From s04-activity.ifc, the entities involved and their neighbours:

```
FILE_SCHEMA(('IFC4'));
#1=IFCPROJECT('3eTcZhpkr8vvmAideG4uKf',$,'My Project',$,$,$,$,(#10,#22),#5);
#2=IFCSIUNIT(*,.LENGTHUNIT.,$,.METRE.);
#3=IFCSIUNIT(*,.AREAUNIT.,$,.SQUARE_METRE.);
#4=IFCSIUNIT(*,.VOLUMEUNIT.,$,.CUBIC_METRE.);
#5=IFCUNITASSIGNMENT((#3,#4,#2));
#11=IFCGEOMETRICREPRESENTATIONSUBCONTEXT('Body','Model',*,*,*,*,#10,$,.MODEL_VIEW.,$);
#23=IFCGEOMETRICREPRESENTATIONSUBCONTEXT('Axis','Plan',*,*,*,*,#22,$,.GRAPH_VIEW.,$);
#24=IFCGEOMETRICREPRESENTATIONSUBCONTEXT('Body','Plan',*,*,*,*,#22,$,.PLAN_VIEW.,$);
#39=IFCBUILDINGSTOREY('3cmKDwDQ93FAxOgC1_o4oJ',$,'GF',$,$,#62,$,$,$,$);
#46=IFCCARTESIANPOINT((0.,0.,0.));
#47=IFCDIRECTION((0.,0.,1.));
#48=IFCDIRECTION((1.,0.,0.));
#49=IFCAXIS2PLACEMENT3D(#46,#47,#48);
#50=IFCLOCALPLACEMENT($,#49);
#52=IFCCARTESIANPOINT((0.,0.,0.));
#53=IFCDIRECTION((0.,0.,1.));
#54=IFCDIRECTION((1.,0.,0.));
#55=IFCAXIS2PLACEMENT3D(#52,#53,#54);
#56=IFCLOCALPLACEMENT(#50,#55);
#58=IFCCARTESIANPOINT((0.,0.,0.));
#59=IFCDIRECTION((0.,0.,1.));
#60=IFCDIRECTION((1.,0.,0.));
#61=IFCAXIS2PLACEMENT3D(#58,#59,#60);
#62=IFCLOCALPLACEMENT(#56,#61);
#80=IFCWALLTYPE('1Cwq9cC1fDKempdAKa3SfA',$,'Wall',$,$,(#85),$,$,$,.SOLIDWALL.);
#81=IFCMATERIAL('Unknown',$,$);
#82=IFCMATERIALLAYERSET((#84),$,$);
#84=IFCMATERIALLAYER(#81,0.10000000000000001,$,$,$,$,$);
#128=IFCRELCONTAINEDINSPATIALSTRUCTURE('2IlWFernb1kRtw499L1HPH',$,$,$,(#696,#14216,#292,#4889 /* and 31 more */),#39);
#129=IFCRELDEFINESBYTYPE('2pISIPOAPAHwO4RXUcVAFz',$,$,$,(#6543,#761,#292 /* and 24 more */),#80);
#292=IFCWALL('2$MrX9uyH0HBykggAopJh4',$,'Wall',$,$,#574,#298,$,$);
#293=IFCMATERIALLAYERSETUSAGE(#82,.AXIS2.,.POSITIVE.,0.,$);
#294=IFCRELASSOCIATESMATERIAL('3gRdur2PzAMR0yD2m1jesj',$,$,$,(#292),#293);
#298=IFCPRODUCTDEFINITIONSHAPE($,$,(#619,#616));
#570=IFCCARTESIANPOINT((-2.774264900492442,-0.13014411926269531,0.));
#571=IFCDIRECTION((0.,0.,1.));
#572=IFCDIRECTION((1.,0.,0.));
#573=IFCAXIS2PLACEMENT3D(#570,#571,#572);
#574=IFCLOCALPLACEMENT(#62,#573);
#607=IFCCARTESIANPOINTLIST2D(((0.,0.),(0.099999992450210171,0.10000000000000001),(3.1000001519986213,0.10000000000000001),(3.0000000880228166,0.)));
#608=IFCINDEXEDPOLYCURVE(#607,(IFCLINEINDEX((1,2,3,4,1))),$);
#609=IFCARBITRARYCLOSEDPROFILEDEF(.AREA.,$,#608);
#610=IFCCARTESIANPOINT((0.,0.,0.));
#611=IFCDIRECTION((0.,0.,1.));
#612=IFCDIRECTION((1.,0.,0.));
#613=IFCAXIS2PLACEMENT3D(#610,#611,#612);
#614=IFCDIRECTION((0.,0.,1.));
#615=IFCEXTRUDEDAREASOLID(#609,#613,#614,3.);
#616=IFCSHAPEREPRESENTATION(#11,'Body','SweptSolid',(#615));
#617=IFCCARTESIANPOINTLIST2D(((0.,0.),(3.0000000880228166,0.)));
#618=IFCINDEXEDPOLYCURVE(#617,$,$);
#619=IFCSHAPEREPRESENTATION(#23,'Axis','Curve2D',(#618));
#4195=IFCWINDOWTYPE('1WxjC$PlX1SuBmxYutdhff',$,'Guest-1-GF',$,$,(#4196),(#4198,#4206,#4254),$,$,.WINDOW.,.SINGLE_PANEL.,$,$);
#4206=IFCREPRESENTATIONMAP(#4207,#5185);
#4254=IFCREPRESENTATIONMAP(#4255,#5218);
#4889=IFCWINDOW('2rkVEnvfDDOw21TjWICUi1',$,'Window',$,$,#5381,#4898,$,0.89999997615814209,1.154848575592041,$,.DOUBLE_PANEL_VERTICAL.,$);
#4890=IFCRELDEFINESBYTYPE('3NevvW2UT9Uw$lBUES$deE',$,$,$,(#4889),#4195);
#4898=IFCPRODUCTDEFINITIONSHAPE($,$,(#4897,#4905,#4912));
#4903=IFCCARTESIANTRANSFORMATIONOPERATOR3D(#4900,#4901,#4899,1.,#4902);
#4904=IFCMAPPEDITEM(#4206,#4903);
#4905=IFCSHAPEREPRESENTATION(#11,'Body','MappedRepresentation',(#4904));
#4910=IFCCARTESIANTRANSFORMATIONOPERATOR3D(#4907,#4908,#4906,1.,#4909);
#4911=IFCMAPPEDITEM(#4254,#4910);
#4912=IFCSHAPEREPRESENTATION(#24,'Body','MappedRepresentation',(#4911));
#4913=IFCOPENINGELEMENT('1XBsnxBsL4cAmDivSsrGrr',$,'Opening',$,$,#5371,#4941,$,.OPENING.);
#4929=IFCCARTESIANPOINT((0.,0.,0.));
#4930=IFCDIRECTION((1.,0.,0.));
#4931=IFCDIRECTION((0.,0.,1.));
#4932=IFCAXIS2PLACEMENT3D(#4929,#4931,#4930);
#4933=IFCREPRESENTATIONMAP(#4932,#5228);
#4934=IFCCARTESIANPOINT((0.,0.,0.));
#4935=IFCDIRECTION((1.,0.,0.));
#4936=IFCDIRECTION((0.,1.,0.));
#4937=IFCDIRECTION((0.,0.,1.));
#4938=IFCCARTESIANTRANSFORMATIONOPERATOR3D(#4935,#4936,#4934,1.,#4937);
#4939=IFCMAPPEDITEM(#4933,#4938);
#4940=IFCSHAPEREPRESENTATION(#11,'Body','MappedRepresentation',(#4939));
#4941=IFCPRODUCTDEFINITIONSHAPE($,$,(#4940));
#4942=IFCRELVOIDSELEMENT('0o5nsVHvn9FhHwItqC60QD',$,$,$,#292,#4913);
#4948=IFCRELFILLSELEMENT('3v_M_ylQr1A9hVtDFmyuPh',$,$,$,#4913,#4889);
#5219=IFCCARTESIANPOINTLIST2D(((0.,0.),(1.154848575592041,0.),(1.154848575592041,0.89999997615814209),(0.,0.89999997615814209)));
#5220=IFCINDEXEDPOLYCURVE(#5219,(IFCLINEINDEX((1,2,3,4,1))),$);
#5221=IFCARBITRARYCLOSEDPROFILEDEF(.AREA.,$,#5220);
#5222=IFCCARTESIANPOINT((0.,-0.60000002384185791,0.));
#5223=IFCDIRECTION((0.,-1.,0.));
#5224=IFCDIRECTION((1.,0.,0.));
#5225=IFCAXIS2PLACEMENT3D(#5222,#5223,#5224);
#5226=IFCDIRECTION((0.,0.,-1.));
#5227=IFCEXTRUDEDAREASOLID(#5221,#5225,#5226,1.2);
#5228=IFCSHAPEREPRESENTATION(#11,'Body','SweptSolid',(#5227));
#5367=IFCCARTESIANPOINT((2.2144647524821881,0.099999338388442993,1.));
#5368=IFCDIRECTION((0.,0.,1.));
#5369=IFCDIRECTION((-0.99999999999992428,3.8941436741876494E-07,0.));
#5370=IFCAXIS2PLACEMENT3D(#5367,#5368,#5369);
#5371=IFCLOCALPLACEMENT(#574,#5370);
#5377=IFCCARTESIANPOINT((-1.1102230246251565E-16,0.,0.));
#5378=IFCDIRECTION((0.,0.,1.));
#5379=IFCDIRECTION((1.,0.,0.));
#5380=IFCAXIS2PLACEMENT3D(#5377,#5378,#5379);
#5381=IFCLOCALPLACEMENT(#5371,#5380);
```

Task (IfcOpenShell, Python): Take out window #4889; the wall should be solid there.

```python
import ifcopenshell
import ifcopenshell.api.feature
import ifcopenshell.api.root
import ifcopenshell.geom
import ifcopenshell.util.shape

model = ifcopenshell.open("s04-activity.ifc")
settings = ifcopenshell.geom.settings()


def volume(element):
    """Net volume in cubic metres, openings subtracted."""
    shape = ifcopenshell.geom.create_shape(settings, element)
    return ifcopenshell.util.shape.get_volume(shape.geometry)


window = model.by_guid("2rkVEnvfDDOw21TjWICUi1")
opening = window.FillsVoids[0].RelatingOpeningElement
wall = opening.VoidsElements[0].RelatingBuildingElement
before = volume(wall)

ifcopenshell.api.root.remove_product(model, product=window)
ifcopenshell.api.feature.remove_feature(model, feature=opening)

after = volume(wall)

print(f"wall volume {before:.3f} -> {after:.3f} m3")

model.write("s04-activity_updated.ifc")
```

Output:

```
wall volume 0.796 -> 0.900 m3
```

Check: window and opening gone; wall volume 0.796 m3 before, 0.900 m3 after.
